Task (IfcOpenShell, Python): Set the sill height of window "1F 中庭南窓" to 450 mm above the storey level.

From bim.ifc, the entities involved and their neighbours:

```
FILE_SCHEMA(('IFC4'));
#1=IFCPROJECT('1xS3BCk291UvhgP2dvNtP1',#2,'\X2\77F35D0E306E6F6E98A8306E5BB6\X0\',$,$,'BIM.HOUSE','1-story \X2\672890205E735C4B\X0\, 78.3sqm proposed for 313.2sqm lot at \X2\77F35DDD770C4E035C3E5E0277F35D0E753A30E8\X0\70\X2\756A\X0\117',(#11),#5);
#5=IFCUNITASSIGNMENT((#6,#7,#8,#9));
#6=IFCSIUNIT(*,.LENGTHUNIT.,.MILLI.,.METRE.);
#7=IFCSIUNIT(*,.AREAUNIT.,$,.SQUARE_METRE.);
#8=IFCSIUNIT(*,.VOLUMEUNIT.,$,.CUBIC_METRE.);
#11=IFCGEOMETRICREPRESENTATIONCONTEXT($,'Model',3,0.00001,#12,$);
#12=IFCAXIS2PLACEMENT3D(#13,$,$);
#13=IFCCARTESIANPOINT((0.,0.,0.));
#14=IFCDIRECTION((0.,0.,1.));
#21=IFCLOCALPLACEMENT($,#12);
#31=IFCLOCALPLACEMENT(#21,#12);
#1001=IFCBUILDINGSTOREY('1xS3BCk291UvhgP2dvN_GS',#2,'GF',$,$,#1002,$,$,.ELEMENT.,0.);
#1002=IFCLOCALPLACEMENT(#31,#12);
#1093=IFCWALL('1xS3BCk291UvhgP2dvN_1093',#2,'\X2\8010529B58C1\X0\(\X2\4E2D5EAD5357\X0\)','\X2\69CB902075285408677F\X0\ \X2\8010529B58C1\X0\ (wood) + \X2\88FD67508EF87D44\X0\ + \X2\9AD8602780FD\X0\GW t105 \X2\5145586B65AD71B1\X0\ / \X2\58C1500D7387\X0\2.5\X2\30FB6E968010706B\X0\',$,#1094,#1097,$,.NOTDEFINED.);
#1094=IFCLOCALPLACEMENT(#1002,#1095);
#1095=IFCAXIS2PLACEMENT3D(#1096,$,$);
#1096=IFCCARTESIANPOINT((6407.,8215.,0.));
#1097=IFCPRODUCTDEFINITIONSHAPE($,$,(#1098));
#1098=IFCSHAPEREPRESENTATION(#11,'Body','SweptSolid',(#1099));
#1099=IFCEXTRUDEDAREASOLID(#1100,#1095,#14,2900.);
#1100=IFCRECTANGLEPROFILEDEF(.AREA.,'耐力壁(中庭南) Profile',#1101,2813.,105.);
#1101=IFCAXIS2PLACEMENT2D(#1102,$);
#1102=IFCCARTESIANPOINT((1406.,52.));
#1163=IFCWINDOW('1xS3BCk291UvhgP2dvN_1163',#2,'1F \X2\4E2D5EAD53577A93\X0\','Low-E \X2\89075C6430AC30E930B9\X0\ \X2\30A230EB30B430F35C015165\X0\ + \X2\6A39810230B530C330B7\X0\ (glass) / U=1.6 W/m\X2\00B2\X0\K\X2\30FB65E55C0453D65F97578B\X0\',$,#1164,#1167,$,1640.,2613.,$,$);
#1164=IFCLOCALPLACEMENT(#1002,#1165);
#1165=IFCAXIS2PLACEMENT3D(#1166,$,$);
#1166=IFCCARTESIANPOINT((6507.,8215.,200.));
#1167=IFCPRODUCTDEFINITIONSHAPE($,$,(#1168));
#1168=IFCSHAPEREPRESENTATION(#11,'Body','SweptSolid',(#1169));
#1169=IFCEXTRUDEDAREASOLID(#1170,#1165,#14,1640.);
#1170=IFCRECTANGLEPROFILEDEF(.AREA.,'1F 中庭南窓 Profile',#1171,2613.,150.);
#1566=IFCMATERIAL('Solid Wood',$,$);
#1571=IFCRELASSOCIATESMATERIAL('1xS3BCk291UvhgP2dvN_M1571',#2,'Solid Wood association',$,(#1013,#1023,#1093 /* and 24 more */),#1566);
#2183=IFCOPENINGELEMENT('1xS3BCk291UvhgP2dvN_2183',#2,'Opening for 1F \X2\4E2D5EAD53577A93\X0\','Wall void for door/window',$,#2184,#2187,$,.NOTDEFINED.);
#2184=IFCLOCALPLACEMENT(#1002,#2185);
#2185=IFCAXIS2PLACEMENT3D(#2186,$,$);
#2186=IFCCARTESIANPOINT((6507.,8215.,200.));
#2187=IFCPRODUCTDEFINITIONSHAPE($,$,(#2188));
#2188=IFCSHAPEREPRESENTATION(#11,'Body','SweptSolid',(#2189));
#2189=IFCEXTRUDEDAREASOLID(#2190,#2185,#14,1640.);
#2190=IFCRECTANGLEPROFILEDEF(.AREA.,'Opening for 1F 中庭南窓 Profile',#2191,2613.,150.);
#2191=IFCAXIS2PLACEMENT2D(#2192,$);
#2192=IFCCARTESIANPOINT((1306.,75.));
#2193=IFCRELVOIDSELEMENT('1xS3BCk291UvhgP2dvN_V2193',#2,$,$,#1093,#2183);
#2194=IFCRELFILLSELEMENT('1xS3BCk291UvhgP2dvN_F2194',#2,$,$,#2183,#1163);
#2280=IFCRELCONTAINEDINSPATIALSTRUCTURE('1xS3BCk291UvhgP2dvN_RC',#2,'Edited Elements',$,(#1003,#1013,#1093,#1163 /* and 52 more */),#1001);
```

```python
import numpy as np
import ifcopenshell
import ifcopenshell.api.geometry
import ifcopenshell.geom
import ifcopenshell.util.element
import ifcopenshell.util.placement
import ifcopenshell.util.shape
import ifcopenshell.util.unit

model = ifcopenshell.open("bim.ifc")
unit_scale = ifcopenshell.util.unit.calculate_unit_scale(model)

window = model.by_guid("1xS3BCk291UvhgP2dvN_1163")
opening = window.FillsVoids[0].RelatingOpeningElement
storey = ifcopenshell.util.element.get_container(window, ifc_class="IfcBuildingStorey")
level = ifcopenshell.util.placement.get_local_placement(storey.ObjectPlacement)[2, 3]

# The opening's origin need not be at the sill, so measure its lowest point.
shape = ifcopenshell.geom.create_shape(ifcopenshell.geom.settings(), opening)
bottom = ifcopenshell.util.shape.get_shape_bottom_elevation(shape, shape.geometry) / unit_scale
dz = level + 0.45 / unit_scale - bottom

shift = np.array([0.0, 0.0, dz])
# The window is not placed relative to its opening, so move both.
for product in (opening, window):
    matrix = ifcopenshell.util.placement.get_local_placement(product.ObjectPlacement)
    matrix[:3, 3] += shift
    ifcopenshell.api.geometry.edit_object_placement(model, product=product, matrix=matrix, is_si=False)

print(f"moved by {dz * unit_scale:+.3f} m")

model.write("bim_updated.ifc")
```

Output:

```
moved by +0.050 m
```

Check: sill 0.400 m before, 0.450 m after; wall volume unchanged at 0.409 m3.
